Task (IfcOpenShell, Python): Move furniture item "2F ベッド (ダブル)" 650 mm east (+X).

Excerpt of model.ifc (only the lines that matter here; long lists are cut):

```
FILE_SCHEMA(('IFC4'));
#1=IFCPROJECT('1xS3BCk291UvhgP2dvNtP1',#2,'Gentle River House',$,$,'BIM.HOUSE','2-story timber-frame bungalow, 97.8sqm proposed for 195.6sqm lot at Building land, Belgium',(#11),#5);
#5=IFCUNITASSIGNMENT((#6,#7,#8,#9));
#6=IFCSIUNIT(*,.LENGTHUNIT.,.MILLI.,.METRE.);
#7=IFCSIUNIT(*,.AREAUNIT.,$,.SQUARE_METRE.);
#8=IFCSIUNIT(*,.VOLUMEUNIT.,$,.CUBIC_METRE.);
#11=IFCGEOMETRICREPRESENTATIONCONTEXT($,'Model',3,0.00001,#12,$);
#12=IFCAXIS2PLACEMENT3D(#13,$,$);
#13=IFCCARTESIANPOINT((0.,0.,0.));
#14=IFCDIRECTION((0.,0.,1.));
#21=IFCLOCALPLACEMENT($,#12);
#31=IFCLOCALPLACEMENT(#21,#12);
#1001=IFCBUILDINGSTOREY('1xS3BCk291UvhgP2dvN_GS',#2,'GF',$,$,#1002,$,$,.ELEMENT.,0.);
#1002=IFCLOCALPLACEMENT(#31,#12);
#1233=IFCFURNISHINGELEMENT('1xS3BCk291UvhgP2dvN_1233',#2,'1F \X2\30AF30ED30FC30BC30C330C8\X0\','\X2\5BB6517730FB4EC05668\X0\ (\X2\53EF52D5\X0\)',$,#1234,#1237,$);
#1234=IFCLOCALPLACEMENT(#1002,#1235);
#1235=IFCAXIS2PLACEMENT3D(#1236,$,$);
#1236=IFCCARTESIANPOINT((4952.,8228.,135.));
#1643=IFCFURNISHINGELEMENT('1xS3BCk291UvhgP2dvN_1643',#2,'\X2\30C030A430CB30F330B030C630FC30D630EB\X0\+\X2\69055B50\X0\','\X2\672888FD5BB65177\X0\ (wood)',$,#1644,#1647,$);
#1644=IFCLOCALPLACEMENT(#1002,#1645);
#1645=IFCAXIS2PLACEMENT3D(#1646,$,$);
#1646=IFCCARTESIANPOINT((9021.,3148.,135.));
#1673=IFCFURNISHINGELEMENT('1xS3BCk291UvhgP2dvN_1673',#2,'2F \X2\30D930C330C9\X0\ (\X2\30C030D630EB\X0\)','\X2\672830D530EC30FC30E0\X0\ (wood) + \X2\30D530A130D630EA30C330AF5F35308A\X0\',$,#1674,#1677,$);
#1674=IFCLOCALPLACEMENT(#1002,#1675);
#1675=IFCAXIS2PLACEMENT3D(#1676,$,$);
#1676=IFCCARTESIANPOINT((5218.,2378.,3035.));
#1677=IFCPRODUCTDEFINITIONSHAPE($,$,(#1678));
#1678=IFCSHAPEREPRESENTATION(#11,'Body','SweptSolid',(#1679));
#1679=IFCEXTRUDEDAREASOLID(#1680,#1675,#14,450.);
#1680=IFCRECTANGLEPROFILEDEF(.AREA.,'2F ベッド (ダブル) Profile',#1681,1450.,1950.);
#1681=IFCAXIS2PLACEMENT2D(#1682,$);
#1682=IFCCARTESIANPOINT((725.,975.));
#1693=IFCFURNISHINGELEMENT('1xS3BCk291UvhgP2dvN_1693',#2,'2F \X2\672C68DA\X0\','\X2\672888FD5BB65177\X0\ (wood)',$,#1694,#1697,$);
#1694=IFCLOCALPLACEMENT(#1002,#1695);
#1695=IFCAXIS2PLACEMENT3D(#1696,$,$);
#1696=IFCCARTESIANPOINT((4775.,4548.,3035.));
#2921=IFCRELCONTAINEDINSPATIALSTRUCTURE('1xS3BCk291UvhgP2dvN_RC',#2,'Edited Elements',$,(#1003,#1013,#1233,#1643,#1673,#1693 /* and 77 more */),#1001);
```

```python
import ifcopenshell
import ifcopenshell.api.geometry
import ifcopenshell.util.placement

model = ifcopenshell.open("model.ifc")

item = model.by_guid("1xS3BCk291UvhgP2dvN_1673")
matrix = ifcopenshell.util.placement.get_local_placement(item.ObjectPlacement)
matrix[0, 3] += 650.0
ifcopenshell.api.geometry.edit_object_placement(model, product=item, matrix=matrix, is_si=False)

print(ifcopenshell.util.placement.get_local_placement(item.ObjectPlacement).round(3) + 0.0)

model.write("model_edited.ifc")
```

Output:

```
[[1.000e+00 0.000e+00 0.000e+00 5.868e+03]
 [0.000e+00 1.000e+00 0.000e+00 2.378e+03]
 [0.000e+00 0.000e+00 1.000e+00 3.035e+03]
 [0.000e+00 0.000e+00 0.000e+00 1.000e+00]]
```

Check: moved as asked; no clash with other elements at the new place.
